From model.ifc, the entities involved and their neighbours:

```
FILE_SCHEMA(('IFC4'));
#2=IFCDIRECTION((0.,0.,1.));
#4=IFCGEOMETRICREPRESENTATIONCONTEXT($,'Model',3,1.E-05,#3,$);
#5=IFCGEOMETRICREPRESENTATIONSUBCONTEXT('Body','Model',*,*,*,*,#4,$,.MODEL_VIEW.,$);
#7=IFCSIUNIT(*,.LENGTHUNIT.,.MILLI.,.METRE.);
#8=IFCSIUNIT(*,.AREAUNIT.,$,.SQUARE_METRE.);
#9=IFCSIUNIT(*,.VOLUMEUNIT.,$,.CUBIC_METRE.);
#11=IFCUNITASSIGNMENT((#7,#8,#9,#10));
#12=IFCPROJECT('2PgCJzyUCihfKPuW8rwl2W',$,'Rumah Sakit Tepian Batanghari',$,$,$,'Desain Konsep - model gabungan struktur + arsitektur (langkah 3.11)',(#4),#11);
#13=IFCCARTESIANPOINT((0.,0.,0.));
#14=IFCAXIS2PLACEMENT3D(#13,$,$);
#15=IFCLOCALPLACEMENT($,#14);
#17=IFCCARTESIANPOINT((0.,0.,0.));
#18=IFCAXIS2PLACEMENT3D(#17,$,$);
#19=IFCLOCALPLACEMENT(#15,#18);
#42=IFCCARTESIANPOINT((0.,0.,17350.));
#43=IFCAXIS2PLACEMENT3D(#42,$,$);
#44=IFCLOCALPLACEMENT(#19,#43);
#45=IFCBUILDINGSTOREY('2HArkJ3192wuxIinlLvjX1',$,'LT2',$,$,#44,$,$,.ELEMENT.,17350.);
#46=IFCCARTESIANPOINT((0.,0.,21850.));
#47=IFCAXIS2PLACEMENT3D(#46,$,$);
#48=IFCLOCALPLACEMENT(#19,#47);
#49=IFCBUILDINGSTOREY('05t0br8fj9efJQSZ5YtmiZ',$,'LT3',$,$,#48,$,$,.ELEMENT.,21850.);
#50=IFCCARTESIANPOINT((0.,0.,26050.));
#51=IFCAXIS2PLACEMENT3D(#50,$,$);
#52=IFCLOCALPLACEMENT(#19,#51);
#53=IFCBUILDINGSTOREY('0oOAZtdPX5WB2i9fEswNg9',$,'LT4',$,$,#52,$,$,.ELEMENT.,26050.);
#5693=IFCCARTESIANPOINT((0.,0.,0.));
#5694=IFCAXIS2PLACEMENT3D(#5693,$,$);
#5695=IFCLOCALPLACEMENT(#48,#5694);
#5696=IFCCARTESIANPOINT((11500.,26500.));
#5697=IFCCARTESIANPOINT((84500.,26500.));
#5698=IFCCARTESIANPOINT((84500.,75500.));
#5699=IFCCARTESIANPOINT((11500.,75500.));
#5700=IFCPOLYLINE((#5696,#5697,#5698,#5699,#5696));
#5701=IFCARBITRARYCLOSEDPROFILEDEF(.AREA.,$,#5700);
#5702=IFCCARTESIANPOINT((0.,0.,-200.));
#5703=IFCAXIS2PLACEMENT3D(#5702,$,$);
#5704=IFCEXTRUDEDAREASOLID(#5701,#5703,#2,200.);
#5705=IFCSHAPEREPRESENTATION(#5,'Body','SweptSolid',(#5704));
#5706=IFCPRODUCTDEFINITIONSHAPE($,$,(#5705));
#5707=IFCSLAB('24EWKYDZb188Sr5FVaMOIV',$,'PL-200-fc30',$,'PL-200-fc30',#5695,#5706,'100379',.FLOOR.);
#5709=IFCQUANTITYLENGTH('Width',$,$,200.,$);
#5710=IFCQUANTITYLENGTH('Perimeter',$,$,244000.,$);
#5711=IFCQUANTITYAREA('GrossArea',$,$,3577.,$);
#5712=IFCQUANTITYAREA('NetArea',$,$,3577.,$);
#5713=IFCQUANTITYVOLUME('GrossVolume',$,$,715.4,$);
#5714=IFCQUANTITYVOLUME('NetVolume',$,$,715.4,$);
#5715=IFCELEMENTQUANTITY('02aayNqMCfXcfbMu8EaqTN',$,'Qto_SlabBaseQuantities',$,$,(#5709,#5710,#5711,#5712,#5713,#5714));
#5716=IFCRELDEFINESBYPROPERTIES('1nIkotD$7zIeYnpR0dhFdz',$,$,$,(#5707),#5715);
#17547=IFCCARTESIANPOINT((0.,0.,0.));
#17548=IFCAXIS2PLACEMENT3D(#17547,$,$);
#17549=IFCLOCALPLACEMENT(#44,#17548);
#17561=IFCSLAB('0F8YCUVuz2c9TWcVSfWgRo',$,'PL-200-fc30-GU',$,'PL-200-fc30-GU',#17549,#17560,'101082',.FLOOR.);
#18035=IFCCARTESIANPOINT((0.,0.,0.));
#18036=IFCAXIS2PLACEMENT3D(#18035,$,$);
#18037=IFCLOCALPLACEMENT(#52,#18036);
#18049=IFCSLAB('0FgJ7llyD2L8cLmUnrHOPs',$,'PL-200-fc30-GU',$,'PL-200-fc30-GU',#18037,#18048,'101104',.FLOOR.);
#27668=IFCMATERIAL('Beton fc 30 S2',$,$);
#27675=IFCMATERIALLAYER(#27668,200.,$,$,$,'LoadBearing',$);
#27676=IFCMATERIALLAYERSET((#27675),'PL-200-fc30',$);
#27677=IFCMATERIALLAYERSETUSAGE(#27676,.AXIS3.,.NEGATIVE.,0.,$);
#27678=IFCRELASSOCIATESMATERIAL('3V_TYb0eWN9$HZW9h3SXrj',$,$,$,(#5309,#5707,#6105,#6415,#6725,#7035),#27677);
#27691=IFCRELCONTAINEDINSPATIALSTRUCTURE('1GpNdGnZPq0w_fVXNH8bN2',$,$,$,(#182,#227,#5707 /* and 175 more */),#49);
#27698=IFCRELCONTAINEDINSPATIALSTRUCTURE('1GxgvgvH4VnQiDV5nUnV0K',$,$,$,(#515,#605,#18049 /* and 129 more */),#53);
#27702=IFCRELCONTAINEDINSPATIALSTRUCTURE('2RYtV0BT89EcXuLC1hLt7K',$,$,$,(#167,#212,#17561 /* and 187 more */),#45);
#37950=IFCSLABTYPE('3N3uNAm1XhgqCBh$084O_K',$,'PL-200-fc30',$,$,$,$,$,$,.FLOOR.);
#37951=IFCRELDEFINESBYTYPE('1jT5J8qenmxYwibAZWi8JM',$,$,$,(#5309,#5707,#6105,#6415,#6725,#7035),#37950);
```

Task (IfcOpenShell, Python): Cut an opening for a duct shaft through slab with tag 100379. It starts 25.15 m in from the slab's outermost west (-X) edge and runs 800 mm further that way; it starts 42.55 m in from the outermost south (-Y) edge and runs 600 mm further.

```python
import numpy as np
import ifcopenshell
import ifcopenshell.api.feature
import ifcopenshell.api.geometry
import ifcopenshell.api.pset
import ifcopenshell.api.root
import ifcopenshell.geom
import ifcopenshell.util.element
import ifcopenshell.util.placement
import ifcopenshell.util.representation
import ifcopenshell.util.shape
import ifcopenshell.util.unit

model = ifcopenshell.open("model.ifc")
unit_scale = ifcopenshell.util.unit.calculate_unit_scale(model)
area_scale = ifcopenshell.util.unit.calculate_unit_scale(model, "AREAUNIT")
volume_scale = ifcopenshell.util.unit.calculate_unit_scale(model, "VOLUMEUNIT")
settings = ifcopenshell.geom.settings()


def volume(element):
    """Net volume in cubic metres, openings subtracted."""
    shape = ifcopenshell.geom.create_shape(settings, element)
    return ifcopenshell.util.shape.get_volume(shape.geometry)


slab = model.by_id(5707)
before = volume(slab)

# Extent in the slab's own axes, in metres. The edges named are its -X and -Y sides.
slab_shape = ifcopenshell.geom.create_shape(settings, slab)
vertices = ifcopenshell.util.shape.get_vertices(slab_shape.geometry)
x_min, y_min, bottom = vertices.min(axis=0)
top = vertices[:, 2].max()

opening = ifcopenshell.api.root.create_entity(model, ifc_class="IfcOpeningElement", name="Duct shaft opening", predefined_type="OPENING")
context = ifcopenshell.util.representation.get_context(model, "Model", "Body", "MODEL_VIEW")
width, depth = 0.8, 0.6
outline = [(0.0, 0.0), (width, 0.0), (width, depth), (0.0, depth), (0.0, 0.0)]
# Overshoot both faces by 50 mm so the cut is clean.
shape = ifcopenshell.api.geometry.add_slab_representation(
    model, context=context, depth=top - bottom + 0.1, polyline=outline
)
ifcopenshell.api.geometry.assign_representation(model, product=opening, representation=shape)

matrix = ifcopenshell.util.placement.get_local_placement(slab.ObjectPlacement)
matrix[:, 3] = matrix @ np.append(np.array([x_min + 25.15, y_min + 42.55, bottom - 0.05]) / unit_scale, 1.0)
ifcopenshell.api.geometry.edit_object_placement(model, product=opening, matrix=matrix, is_si=False)
ifcopenshell.api.feature.add_feature(model, feature=opening, element=slab)

after = volume(slab)

# Update the slab's stored quantities.
qto = model.by_id(ifcopenshell.util.element.get_pset(slab, "Qto_SlabBaseQuantities", should_inherit=False)["id"])
ifcopenshell.api.pset.edit_qto(model, qto=qto, properties={
    "NetArea": after / (top - bottom) / area_scale,
    "NetVolume": after / volume_scale,
})

print(f"slab volume {before:.3f} -> {after:.3f} m3")

model.write("model_v2.ifc")
```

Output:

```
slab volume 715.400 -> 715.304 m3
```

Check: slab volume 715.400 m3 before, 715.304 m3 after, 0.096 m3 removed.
